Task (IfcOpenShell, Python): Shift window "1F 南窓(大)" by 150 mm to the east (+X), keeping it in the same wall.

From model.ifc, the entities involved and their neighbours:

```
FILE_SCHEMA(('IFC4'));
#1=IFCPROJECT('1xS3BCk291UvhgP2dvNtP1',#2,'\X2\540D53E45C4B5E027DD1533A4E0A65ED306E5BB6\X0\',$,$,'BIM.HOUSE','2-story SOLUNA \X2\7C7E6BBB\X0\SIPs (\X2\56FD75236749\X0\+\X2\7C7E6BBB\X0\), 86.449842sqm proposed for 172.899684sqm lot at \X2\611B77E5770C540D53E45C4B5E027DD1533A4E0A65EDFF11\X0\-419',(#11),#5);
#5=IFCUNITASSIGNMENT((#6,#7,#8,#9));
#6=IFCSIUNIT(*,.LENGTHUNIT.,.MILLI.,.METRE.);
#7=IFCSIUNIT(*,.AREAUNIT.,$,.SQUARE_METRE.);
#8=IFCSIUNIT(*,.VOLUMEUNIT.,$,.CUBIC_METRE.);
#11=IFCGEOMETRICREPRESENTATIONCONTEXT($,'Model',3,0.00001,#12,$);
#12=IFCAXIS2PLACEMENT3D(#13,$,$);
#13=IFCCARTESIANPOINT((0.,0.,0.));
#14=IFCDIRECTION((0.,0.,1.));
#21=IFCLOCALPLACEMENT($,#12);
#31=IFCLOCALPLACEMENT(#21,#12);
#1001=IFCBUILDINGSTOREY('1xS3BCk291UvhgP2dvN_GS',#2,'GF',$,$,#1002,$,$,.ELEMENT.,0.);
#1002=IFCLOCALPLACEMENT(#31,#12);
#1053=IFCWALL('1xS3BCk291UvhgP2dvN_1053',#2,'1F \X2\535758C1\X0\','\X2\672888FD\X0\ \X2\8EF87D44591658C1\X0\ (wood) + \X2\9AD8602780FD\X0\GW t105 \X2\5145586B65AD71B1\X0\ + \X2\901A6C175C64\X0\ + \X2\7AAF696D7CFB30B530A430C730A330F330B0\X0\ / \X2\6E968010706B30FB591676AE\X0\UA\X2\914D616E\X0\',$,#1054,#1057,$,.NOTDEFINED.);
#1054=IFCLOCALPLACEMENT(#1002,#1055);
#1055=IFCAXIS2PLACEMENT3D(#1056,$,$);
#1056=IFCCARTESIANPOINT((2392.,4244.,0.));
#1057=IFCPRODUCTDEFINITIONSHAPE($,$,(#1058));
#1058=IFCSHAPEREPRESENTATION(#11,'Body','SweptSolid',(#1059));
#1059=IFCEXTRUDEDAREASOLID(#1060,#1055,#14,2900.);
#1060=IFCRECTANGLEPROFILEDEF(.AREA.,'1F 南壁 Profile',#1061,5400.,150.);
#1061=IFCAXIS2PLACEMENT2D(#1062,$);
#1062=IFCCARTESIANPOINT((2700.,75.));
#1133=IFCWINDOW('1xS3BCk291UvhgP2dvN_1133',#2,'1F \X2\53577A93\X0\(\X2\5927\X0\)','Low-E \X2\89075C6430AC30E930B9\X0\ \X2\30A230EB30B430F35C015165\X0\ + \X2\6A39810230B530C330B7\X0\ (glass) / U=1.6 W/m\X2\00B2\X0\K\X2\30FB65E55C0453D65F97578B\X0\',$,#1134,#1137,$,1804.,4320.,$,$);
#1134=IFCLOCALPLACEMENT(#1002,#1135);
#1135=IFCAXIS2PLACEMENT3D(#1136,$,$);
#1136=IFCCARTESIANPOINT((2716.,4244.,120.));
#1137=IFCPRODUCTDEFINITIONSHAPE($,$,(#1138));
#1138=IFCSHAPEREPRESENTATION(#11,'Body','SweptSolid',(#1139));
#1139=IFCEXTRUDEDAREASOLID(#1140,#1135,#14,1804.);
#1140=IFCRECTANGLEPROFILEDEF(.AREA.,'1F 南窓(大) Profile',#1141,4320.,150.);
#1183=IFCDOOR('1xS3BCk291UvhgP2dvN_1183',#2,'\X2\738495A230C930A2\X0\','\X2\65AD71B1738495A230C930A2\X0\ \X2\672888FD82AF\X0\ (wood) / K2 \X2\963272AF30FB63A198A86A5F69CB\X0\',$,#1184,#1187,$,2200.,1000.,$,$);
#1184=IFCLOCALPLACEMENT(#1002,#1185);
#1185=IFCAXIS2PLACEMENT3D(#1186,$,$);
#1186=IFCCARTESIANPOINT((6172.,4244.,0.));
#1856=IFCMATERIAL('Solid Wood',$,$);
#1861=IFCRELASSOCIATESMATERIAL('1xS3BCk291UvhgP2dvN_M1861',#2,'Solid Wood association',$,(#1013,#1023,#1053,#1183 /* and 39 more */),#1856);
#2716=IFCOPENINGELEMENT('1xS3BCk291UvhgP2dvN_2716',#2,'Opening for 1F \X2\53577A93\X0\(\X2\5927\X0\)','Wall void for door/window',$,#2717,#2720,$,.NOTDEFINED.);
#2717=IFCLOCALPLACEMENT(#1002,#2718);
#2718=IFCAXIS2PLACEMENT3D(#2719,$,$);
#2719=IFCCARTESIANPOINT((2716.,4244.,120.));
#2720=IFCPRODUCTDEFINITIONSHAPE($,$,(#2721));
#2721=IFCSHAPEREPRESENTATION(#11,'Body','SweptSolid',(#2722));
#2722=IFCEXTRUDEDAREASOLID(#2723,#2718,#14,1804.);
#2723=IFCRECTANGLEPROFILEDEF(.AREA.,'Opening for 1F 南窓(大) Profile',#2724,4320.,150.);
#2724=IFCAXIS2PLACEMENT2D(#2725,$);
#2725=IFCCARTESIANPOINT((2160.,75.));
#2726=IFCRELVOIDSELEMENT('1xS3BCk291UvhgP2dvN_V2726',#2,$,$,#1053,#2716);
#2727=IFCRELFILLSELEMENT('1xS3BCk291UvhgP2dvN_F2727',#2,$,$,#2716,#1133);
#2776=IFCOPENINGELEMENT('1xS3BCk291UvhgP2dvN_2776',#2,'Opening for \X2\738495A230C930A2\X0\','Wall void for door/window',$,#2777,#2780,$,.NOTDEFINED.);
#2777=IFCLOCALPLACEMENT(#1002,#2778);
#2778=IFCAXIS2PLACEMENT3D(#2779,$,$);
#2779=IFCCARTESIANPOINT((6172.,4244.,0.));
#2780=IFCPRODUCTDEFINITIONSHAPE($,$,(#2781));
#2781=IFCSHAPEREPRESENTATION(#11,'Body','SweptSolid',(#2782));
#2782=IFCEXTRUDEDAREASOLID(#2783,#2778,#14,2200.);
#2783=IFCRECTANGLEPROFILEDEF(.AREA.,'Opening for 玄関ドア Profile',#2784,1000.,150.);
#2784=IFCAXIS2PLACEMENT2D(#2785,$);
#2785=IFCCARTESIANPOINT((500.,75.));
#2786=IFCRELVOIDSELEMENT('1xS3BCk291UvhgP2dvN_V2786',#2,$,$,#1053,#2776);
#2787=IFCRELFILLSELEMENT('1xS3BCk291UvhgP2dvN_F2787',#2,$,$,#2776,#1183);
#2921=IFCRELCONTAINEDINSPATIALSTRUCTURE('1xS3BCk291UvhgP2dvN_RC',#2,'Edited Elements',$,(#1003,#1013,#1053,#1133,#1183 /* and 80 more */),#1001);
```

```python
import ifcopenshell
import ifcopenshell.api.geometry
import ifcopenshell.util.placement

model = ifcopenshell.open("model.ifc")

window = model.by_guid("1xS3BCk291UvhgP2dvN_1133")
opening = window.FillsVoids[0].RelatingOpeningElement
wall = opening.VoidsElements[0].RelatingBuildingElement

wall_matrix = ifcopenshell.util.placement.get_local_placement(wall.ObjectPlacement)
shift = wall_matrix[:3, 0] * 150.0
before = ifcopenshell.util.placement.get_local_placement(window.ObjectPlacement)[:3, 3].copy()

# The window is not placed relative to its opening, so move both.
for product in (opening, window):
    matrix = ifcopenshell.util.placement.get_local_placement(product.ObjectPlacement)
    matrix[:3, 3] += shift
    ifcopenshell.api.geometry.edit_object_placement(model, product=product, matrix=matrix, is_si=False)

after = ifcopenshell.util.placement.get_local_placement(window.ObjectPlacement)[:3, 3]
print("window moved by", (after - before).round(3) + 0.0)

model.write("model_rev.ifc")
```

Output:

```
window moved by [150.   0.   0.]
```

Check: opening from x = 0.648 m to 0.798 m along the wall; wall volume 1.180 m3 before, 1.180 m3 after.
